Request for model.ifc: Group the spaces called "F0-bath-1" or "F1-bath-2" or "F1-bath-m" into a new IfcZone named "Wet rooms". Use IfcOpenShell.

First a look at what the model holds.

```python
import ifcopenshell

model = ifcopenshell.open("model.ifc")
print(model.schema)
seen = {}
for space in model.by_type("IfcSpace"):
    seen[space.LongName] = seen.get(space.LongName, 0) + 1
for name, count in sorted(seen.items(), key=str):
    print(count, "x", name)
print("zones:", [z.Name for z in model.by_type("IfcZone")][:20])
```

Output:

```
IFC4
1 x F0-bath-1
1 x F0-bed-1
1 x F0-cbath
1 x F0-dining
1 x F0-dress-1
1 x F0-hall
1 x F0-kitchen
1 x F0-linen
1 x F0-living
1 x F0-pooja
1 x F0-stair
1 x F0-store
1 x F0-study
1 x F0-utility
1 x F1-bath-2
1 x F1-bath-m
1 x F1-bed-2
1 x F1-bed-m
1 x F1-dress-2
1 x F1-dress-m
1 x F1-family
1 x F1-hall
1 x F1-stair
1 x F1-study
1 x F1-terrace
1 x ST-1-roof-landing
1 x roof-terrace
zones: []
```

```python
import ifcopenshell
import ifcopenshell.api.group
import ifcopenshell.api.root

model = ifcopenshell.open("model.ifc")

names = {"F0-bath-1", "F1-bath-2", "F1-bath-m"}
spaces = [s for s in model.by_type("IfcSpace") if s.LongName in names]

zone = ifcopenshell.api.root.create_entity(model, ifc_class="IfcZone", name="Wet rooms")
ifcopenshell.api.group.assign_group(model, products=spaces, group=zone)
print(len(spaces), "spaces in", zone.Name)

model.write("model_v2.ifc")
```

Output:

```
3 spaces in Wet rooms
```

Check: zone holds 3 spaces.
